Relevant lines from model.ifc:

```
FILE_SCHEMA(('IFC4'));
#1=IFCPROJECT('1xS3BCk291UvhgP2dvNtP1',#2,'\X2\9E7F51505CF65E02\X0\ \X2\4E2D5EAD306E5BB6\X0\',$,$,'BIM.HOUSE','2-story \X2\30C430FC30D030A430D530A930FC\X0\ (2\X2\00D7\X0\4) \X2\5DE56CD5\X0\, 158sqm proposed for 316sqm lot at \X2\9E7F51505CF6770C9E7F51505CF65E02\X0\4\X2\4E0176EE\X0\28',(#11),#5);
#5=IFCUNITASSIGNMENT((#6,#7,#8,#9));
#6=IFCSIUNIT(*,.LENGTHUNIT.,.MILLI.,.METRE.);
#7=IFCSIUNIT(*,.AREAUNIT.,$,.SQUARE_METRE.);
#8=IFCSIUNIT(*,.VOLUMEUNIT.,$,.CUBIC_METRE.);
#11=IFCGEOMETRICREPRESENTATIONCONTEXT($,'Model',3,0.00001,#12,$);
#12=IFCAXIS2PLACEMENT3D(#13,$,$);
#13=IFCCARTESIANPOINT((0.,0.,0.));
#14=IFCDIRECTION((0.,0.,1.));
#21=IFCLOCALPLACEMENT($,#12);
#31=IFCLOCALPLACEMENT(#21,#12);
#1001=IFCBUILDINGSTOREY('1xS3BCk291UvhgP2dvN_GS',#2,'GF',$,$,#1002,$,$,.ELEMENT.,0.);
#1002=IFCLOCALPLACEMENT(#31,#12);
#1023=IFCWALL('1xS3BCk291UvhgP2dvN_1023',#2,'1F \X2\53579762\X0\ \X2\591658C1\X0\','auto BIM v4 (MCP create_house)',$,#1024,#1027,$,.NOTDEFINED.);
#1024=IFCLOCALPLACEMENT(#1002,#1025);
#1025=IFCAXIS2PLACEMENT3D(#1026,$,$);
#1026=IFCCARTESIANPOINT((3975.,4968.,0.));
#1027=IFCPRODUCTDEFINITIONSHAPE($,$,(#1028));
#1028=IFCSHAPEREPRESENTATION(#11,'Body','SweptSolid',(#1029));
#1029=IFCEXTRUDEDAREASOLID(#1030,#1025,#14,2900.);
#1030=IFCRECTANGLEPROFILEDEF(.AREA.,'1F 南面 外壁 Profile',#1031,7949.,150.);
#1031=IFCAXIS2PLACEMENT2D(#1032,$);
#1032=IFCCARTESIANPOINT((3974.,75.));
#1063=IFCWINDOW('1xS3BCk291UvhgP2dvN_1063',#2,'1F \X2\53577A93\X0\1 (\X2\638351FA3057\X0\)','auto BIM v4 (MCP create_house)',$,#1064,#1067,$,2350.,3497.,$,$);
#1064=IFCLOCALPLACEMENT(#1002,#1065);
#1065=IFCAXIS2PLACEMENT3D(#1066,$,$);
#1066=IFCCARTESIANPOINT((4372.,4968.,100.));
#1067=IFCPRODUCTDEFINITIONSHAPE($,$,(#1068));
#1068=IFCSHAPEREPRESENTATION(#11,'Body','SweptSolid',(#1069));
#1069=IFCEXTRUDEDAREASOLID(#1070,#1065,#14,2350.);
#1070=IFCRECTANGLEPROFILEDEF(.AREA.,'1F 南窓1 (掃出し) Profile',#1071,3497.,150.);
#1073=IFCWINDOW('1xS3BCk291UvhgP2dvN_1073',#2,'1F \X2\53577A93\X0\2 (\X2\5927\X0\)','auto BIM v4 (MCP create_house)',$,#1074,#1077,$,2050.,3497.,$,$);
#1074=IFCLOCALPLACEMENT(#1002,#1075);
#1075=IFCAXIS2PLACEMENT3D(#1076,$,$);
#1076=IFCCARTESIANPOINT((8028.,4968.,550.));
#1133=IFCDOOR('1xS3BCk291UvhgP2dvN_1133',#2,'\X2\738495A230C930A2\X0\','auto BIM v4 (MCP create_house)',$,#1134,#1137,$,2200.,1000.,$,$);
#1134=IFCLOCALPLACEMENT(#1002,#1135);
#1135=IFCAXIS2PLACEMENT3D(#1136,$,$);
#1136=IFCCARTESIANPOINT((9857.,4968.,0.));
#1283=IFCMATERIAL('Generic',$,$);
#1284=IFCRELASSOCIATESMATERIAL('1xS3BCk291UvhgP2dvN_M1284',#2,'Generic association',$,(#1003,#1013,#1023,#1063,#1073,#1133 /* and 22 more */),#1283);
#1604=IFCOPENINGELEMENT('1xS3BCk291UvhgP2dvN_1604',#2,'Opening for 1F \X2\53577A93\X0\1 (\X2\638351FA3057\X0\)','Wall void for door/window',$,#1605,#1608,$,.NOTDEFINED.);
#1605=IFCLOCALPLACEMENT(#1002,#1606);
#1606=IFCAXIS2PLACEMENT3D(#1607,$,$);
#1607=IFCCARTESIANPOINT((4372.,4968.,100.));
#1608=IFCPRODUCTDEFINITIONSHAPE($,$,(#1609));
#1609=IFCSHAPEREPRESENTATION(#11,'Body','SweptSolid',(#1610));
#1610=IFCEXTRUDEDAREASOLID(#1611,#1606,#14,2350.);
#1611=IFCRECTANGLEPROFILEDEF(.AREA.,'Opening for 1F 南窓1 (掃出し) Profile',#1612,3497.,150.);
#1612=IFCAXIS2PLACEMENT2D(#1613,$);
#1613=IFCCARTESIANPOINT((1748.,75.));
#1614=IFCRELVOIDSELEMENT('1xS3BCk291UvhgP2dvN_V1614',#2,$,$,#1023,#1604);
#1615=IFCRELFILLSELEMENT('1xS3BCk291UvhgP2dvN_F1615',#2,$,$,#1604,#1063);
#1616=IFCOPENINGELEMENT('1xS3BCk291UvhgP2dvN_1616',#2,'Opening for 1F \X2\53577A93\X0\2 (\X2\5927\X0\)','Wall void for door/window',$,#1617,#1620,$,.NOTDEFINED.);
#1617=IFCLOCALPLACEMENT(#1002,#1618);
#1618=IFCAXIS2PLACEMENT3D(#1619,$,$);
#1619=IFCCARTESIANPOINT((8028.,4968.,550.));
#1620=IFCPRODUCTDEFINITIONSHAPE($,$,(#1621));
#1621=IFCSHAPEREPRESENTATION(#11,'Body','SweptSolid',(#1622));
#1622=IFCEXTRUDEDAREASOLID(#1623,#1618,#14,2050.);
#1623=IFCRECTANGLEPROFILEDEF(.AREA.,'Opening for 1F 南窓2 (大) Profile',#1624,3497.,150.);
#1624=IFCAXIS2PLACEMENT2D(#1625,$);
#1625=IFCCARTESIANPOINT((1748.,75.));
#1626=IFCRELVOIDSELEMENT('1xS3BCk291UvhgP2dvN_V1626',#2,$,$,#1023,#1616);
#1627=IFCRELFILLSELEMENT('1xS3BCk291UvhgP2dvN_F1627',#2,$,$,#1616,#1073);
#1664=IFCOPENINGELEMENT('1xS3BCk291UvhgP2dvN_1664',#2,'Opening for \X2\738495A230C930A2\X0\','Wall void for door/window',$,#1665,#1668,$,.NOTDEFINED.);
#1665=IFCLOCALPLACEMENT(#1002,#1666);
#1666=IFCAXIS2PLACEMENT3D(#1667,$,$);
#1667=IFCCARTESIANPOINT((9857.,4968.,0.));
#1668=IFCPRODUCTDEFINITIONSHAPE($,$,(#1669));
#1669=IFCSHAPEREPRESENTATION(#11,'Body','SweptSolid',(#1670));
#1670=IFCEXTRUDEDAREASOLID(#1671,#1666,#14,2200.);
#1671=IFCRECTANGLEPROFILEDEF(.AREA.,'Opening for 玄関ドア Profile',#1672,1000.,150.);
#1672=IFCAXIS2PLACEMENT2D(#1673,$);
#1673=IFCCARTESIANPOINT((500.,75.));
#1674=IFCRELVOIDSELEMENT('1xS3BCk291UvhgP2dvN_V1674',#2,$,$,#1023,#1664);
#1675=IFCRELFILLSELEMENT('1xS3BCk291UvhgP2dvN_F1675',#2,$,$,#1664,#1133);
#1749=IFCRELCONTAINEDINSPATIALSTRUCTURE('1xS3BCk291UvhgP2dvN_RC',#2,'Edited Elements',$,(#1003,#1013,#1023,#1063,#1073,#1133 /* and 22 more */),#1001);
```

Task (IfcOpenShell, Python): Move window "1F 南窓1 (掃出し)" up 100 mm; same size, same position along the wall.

```python
import numpy as np
import ifcopenshell
import ifcopenshell.api.geometry
import ifcopenshell.util.placement
import ifcopenshell.util.unit

model = ifcopenshell.open("model.ifc")
unit_scale = ifcopenshell.util.unit.calculate_unit_scale(model)

window = model.by_id(1063)
opening = window.FillsVoids[0].RelatingOpeningElement
dz = 100.0

shift = np.array([0.0, 0.0, dz])
# The window is not placed relative to its opening, so move both.
for product in (opening, window):
    matrix = ifcopenshell.util.placement.get_local_placement(product.ObjectPlacement)
    matrix[:3, 3] += shift
    ifcopenshell.api.geometry.edit_object_placement(model, product=product, matrix=matrix, is_si=False)

print(f"moved by {dz * unit_scale:+.3f} m")

model.write("model_edited.ifc")
```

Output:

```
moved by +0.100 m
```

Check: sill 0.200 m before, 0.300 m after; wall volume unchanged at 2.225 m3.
